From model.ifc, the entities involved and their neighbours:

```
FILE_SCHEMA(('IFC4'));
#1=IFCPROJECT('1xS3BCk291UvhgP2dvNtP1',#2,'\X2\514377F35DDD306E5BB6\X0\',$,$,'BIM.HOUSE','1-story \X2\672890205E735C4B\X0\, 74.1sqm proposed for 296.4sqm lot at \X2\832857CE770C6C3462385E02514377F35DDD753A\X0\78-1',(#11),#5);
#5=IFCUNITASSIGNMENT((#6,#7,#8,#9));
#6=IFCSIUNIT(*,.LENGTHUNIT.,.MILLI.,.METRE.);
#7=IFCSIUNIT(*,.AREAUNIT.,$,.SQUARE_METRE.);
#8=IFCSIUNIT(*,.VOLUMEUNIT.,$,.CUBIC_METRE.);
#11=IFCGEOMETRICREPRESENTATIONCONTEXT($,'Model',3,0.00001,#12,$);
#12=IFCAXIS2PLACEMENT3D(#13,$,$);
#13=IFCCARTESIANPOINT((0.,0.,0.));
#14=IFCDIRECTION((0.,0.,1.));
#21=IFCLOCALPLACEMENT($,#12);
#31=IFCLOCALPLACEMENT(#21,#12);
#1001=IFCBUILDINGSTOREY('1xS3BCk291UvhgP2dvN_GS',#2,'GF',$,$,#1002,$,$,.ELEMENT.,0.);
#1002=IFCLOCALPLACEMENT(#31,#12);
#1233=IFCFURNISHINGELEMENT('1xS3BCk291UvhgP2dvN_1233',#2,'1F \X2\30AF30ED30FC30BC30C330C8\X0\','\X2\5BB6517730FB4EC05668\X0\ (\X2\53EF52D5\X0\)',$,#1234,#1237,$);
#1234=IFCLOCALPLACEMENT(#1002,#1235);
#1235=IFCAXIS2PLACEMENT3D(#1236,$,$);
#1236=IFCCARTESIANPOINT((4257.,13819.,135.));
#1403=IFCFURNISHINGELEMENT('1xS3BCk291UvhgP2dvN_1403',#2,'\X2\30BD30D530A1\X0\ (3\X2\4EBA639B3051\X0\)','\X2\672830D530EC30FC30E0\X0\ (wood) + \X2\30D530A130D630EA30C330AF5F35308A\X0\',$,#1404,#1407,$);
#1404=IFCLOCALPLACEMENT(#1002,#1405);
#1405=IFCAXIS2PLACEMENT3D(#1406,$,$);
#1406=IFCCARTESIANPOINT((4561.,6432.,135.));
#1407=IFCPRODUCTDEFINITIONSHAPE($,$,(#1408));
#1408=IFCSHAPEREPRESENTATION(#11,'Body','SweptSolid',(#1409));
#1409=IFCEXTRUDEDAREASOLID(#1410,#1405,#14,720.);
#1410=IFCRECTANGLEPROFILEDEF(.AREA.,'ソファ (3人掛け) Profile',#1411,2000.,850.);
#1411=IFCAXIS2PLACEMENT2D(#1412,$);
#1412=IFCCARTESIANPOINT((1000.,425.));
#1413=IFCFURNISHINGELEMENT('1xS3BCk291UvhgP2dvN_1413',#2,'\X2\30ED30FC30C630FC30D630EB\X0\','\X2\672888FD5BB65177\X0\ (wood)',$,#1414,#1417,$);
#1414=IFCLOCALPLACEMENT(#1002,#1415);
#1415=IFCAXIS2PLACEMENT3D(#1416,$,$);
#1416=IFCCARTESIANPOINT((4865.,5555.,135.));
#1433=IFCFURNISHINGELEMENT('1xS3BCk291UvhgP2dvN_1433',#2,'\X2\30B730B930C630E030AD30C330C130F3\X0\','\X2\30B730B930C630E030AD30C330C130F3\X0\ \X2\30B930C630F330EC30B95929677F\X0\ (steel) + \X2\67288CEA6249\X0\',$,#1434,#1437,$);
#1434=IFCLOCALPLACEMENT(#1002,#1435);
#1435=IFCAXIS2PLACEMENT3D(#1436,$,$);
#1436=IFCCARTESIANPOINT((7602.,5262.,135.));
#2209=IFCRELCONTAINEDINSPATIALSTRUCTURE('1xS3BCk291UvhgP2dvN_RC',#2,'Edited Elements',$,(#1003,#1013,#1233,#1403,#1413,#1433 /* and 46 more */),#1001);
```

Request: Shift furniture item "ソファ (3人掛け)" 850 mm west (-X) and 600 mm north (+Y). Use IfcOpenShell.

```python
import ifcopenshell
import ifcopenshell.api.geometry
import ifcopenshell.util.placement

model = ifcopenshell.open("model.ifc")

item = model.by_id(1403)
matrix = ifcopenshell.util.placement.get_local_placement(item.ObjectPlacement)
matrix[0, 3] -= 850.0
matrix[1, 3] += 600.0
ifcopenshell.api.geometry.edit_object_placement(model, product=item, matrix=matrix, is_si=False)

print(ifcopenshell.util.placement.get_local_placement(item.ObjectPlacement).round(3) + 0.0)

model.write("model_rev.ifc")
```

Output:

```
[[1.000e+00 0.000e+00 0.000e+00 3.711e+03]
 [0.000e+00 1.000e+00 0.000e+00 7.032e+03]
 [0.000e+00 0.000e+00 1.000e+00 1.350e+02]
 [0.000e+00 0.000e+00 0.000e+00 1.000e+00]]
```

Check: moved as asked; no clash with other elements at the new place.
